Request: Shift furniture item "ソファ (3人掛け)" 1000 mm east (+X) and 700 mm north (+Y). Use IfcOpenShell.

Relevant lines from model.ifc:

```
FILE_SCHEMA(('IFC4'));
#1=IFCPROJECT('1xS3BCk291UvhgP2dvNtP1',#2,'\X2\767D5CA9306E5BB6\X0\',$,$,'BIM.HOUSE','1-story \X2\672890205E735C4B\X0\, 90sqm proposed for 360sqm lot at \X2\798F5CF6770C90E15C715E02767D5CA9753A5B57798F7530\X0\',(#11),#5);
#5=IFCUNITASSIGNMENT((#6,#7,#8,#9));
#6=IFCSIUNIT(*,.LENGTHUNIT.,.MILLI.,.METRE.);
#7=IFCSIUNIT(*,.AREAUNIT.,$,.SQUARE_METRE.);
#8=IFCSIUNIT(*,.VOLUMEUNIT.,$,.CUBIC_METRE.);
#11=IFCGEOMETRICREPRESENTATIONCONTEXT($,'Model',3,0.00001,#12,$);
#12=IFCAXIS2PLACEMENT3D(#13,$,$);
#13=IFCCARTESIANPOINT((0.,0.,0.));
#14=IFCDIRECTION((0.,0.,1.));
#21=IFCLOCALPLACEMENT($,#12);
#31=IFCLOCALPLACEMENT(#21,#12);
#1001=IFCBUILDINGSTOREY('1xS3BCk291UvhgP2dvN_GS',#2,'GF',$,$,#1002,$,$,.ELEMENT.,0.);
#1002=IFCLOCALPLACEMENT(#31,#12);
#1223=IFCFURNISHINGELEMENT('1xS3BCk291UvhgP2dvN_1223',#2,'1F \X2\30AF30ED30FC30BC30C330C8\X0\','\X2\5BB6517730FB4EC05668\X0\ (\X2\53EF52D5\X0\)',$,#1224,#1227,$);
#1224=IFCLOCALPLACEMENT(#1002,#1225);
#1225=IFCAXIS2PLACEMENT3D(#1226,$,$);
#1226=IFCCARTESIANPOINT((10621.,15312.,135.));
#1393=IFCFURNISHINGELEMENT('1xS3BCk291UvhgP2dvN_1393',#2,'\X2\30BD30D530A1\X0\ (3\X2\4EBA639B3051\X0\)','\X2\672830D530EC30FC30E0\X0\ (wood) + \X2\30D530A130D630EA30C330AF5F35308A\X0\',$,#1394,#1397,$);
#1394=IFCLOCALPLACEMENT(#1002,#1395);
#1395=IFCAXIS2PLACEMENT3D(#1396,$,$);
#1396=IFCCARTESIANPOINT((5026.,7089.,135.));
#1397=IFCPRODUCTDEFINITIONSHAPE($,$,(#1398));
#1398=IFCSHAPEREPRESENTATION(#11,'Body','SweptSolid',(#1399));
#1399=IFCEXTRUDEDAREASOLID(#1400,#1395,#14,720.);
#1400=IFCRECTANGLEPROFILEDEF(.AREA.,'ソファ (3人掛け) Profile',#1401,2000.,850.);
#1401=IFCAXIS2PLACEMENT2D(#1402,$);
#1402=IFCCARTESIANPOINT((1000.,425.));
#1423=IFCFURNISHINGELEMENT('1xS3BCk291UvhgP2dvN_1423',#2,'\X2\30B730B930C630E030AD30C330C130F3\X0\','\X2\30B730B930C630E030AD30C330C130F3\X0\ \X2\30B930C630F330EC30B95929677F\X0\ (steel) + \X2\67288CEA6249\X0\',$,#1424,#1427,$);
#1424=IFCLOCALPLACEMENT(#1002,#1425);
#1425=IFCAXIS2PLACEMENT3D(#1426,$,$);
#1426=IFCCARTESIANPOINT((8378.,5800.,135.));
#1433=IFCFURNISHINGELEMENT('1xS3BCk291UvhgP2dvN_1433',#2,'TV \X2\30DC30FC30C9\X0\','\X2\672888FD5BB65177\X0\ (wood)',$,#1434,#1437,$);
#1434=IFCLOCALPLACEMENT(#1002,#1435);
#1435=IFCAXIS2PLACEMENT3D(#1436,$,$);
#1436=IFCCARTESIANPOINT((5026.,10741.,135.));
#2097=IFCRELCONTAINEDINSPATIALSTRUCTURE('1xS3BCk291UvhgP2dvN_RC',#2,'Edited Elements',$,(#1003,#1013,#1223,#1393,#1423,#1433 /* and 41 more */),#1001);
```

```python
import ifcopenshell
import ifcopenshell.api.geometry
import ifcopenshell.util.placement
import ifcopenshell.util.unit

model = ifcopenshell.open("model.ifc")
unit_scale = ifcopenshell.util.unit.calculate_unit_scale(model)

item = model.by_guid("1xS3BCk291UvhgP2dvN_1393")
matrix = ifcopenshell.util.placement.get_local_placement(item.ObjectPlacement)
matrix[0, 3] += 1 / unit_scale
matrix[1, 3] += 0.7 / unit_scale
ifcopenshell.api.geometry.edit_object_placement(model, product=item, matrix=matrix, is_si=False)

print(ifcopenshell.util.placement.get_local_placement(item.ObjectPlacement).round(3) + 0.0)

model.write("model_rev.ifc")
```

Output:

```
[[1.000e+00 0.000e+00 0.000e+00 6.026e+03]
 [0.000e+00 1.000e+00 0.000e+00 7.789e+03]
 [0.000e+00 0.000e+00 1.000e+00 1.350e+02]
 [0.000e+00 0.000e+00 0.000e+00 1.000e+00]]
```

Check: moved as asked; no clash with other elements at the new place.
